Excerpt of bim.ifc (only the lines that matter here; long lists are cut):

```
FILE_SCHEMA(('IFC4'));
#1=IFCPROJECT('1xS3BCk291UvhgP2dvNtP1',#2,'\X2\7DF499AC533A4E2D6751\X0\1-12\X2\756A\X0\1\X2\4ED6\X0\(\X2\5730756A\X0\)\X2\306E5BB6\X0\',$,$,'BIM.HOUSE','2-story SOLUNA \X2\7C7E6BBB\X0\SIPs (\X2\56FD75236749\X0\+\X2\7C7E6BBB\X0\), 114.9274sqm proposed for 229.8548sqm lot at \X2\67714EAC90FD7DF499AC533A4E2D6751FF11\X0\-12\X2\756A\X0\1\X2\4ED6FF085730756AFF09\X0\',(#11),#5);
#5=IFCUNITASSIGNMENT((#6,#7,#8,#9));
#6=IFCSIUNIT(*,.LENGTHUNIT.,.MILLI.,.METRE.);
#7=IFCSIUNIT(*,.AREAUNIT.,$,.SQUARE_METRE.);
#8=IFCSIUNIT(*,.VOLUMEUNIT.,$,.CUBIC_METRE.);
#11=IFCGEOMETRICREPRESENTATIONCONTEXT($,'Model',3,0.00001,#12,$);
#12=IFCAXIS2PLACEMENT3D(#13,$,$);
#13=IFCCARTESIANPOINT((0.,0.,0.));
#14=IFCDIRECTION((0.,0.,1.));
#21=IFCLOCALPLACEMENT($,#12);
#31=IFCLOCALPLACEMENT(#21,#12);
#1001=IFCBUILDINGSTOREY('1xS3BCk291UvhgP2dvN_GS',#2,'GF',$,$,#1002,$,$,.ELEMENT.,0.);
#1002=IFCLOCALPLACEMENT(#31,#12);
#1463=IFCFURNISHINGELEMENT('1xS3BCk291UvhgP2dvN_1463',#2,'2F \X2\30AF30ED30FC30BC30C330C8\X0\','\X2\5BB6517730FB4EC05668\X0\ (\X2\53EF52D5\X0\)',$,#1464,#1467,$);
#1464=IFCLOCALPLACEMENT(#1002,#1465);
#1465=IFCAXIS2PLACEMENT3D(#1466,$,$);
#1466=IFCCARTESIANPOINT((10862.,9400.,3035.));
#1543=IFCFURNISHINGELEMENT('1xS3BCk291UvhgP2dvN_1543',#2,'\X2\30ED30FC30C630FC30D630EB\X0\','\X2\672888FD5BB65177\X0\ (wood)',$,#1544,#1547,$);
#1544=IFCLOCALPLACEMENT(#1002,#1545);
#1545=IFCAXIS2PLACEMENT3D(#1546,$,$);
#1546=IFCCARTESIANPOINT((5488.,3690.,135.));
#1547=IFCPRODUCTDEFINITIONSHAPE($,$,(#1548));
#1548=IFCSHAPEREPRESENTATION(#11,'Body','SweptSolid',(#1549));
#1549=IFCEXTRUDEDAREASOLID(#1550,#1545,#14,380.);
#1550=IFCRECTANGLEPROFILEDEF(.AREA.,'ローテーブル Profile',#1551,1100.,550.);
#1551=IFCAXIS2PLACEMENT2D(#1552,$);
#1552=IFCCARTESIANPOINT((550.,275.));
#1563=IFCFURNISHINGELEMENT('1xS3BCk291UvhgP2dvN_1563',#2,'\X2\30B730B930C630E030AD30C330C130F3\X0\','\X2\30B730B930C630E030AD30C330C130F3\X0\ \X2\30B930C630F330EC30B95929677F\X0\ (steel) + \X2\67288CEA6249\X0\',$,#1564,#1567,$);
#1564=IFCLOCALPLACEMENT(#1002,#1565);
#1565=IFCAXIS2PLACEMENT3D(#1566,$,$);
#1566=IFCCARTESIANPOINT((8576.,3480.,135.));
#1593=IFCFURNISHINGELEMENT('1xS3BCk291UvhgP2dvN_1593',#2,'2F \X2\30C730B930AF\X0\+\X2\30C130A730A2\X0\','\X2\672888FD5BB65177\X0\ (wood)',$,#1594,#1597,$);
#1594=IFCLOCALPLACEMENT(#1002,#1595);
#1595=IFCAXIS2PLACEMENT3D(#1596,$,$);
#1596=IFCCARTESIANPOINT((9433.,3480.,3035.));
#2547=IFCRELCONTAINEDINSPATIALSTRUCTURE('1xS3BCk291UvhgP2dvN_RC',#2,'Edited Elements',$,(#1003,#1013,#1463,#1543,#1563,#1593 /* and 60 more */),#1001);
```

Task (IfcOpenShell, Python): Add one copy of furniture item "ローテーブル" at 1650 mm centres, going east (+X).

```python
import numpy as np
import ifcopenshell
import ifcopenshell.api.geometry
import ifcopenshell.api.root
import ifcopenshell.util.element
import ifcopenshell.util.placement

model = ifcopenshell.open("bim.ifc")


def reuse_history(source, copy):
    """copy_class also copies each property set's owner history, people and application; keep the originals."""
    for rel in copy.IsDefinedBy:
        if rel.is_a("IfcRelDefinesByProperties") and (history := rel.RelatingPropertyDefinition.OwnerHistory):
            rel.RelatingPropertyDefinition.OwnerHistory = source.OwnerHistory
            ifcopenshell.util.element.remove_deep2(model, history)


source = model.by_id(1543)
base = ifcopenshell.util.placement.get_local_placement(source.ObjectPlacement)
step = np.array([1.0, 0.0, 0.0]) * 1650.0

for i in range(1, 2):
    copy = ifcopenshell.api.root.copy_class(model, product=source)
    copy.Representation = ifcopenshell.util.element.copy_deep(
        model, source.Representation, exclude=["IfcGeometricRepresentationContext", "IfcRepresentationMap"]
    )
    reuse_history(source, copy)
    matrix = base.copy()
    matrix[:3, 3] += i * step
    print("added at", matrix[:3, 3].round(3) + 0.0)
    ifcopenshell.api.geometry.edit_object_placement(model, product=copy, matrix=matrix, is_si=False)

model.write("bim_v2.ifc")
```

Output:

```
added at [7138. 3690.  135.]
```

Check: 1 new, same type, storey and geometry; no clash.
